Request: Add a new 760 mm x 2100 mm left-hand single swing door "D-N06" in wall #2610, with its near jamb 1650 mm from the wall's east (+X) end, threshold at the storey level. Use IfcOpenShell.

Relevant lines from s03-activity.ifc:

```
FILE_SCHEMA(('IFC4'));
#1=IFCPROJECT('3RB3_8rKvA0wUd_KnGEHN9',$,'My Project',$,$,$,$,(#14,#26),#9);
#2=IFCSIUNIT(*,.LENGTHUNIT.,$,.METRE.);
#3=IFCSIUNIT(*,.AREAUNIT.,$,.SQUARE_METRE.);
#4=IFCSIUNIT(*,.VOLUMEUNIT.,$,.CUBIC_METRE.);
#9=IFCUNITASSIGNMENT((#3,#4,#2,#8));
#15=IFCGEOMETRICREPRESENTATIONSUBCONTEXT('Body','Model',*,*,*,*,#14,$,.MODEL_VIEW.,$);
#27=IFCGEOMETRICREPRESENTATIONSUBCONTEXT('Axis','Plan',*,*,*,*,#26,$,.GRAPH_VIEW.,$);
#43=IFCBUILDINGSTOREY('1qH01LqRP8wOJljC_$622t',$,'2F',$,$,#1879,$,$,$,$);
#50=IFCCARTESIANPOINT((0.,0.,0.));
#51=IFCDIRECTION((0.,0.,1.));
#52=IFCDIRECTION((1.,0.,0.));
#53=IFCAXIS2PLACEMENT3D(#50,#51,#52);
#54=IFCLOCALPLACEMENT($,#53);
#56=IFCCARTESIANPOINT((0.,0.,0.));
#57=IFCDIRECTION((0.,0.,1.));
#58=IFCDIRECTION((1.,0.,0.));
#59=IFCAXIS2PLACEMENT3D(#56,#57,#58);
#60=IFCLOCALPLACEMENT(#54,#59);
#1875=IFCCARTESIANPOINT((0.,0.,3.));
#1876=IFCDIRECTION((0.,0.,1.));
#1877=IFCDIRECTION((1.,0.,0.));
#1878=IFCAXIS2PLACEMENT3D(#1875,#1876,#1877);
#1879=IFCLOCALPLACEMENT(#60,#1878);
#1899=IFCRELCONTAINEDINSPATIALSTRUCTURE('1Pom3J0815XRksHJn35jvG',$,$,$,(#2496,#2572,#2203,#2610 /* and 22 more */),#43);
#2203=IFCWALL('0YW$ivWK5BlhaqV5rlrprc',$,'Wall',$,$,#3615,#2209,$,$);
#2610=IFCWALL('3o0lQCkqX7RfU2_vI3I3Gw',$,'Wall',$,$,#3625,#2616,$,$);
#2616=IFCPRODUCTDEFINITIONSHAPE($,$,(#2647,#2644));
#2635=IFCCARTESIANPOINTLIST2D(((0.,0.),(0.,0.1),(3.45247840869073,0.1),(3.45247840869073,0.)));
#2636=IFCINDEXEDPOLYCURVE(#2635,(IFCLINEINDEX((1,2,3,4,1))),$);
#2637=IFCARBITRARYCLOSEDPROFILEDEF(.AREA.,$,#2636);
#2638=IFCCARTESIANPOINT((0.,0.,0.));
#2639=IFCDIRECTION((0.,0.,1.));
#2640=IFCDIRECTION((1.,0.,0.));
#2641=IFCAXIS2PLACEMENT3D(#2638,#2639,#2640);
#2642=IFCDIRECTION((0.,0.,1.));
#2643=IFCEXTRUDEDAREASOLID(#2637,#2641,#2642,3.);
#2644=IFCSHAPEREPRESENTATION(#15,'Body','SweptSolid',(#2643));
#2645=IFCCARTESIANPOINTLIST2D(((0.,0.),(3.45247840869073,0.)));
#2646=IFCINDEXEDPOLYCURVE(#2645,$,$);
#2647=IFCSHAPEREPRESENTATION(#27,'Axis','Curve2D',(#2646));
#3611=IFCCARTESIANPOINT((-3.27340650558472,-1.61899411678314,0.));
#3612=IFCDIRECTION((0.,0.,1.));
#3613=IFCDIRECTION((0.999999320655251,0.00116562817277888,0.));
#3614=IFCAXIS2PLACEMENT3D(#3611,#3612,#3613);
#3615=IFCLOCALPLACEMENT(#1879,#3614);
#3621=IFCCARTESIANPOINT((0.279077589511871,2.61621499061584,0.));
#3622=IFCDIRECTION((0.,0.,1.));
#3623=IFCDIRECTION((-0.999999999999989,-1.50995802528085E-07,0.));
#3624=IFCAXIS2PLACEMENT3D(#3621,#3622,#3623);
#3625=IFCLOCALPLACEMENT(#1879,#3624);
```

```python
import numpy as np
import ifcopenshell
import ifcopenshell.api.feature
import ifcopenshell.api.geometry
import ifcopenshell.api.root
import ifcopenshell.api.spatial
import ifcopenshell.geom
import ifcopenshell.util.element
import ifcopenshell.util.placement
import ifcopenshell.util.representation
import ifcopenshell.util.shape
import ifcopenshell.util.unit

model = ifcopenshell.open("s03-activity.ifc")
unit_scale = ifcopenshell.util.unit.calculate_unit_scale(model)
settings = ifcopenshell.geom.settings()


def volume(element):
    """Net volume in cubic metres, openings subtracted."""
    shape = ifcopenshell.geom.create_shape(settings, element)
    return ifcopenshell.util.shape.get_volume(shape.geometry)


wall = model.by_guid("3o0lQCkqX7RfU2_vI3I3Gw")
storey = ifcopenshell.util.element.get_container(wall, ifc_class="IfcBuildingStorey")
context = ifcopenshell.util.representation.get_context(model, "Model", "Body", "MODEL_VIEW")
before = volume(wall)

width, height, from_end, sill = 0.76, 2.1, 1.65, 0.0  # metres

# The wall runs along its own X axis, and the end named is its -X end.
wall_shape = ifcopenshell.geom.create_shape(settings, wall)
x, y, z = ifcopenshell.util.shape.get_vertices(wall_shape.geometry).T
start = x.min() + from_end
face, thickness = float(y.min()), float(y.max() - y.min())
wall_matrix = ifcopenshell.util.placement.get_local_placement(wall.ObjectPlacement)
level = ifcopenshell.util.placement.get_local_placement(storey.ObjectPlacement)[2, 3]


def in_wall(x, y):
    """Placement at x, y metres in the wall's axes, at sill height."""
    matrix = wall_matrix.copy()
    matrix[:, 3] = wall_matrix @ np.array([x / unit_scale, y / unit_scale, 0.0, 1.0])
    matrix[2, 3] = level + sill / unit_scale
    return matrix


# Opening: a box that overshoots both wall faces by 50 mm.
opening = ifcopenshell.api.root.create_entity(model, ifc_class="IfcOpeningElement", predefined_type="OPENING")
box = ifcopenshell.api.geometry.add_wall_representation(
    model, context=context, length=width, height=height, thickness=thickness + 0.1
)
ifcopenshell.api.geometry.assign_representation(model, product=opening, representation=box)
ifcopenshell.api.geometry.edit_object_placement(model, product=opening, matrix=in_wall(start, face - 0.05), is_si=False)
ifcopenshell.api.feature.add_feature(model, feature=opening, element=wall)

door = ifcopenshell.api.root.create_entity(model, ifc_class="IfcDoor", name="D-N06", predefined_type="DOOR")
door.OverallWidth, door.OverallHeight = width / unit_scale, height / unit_scale
door.OperationType = "SINGLE_SWING_LEFT"
body = ifcopenshell.api.geometry.add_door_representation(
    model,
    context=context,
    overall_width=door.OverallWidth,
    overall_height=door.OverallHeight,
    operation_type="SINGLE_SWING_LEFT",
    lining_properties={"LiningDepth": thickness / unit_scale, "ThresholdDepth": thickness / unit_scale},
)
ifcopenshell.api.geometry.assign_representation(model, product=door, representation=body)
ifcopenshell.api.spatial.assign_container(model, products=[door], relating_structure=storey)
ifcopenshell.api.feature.add_filling(model, opening=opening, element=door)

# The lining spans the wall, so the door starts at the wall face.
ifcopenshell.api.geometry.edit_object_placement(model, product=door, matrix=in_wall(start, face), is_si=False)

after = volume(wall)

print(f"wall volume {before:.3f} -> {after:.3f} m3")

model.write("s03-activity_updated.ifc")
```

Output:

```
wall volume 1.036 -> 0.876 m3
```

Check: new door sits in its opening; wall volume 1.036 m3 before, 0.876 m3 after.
